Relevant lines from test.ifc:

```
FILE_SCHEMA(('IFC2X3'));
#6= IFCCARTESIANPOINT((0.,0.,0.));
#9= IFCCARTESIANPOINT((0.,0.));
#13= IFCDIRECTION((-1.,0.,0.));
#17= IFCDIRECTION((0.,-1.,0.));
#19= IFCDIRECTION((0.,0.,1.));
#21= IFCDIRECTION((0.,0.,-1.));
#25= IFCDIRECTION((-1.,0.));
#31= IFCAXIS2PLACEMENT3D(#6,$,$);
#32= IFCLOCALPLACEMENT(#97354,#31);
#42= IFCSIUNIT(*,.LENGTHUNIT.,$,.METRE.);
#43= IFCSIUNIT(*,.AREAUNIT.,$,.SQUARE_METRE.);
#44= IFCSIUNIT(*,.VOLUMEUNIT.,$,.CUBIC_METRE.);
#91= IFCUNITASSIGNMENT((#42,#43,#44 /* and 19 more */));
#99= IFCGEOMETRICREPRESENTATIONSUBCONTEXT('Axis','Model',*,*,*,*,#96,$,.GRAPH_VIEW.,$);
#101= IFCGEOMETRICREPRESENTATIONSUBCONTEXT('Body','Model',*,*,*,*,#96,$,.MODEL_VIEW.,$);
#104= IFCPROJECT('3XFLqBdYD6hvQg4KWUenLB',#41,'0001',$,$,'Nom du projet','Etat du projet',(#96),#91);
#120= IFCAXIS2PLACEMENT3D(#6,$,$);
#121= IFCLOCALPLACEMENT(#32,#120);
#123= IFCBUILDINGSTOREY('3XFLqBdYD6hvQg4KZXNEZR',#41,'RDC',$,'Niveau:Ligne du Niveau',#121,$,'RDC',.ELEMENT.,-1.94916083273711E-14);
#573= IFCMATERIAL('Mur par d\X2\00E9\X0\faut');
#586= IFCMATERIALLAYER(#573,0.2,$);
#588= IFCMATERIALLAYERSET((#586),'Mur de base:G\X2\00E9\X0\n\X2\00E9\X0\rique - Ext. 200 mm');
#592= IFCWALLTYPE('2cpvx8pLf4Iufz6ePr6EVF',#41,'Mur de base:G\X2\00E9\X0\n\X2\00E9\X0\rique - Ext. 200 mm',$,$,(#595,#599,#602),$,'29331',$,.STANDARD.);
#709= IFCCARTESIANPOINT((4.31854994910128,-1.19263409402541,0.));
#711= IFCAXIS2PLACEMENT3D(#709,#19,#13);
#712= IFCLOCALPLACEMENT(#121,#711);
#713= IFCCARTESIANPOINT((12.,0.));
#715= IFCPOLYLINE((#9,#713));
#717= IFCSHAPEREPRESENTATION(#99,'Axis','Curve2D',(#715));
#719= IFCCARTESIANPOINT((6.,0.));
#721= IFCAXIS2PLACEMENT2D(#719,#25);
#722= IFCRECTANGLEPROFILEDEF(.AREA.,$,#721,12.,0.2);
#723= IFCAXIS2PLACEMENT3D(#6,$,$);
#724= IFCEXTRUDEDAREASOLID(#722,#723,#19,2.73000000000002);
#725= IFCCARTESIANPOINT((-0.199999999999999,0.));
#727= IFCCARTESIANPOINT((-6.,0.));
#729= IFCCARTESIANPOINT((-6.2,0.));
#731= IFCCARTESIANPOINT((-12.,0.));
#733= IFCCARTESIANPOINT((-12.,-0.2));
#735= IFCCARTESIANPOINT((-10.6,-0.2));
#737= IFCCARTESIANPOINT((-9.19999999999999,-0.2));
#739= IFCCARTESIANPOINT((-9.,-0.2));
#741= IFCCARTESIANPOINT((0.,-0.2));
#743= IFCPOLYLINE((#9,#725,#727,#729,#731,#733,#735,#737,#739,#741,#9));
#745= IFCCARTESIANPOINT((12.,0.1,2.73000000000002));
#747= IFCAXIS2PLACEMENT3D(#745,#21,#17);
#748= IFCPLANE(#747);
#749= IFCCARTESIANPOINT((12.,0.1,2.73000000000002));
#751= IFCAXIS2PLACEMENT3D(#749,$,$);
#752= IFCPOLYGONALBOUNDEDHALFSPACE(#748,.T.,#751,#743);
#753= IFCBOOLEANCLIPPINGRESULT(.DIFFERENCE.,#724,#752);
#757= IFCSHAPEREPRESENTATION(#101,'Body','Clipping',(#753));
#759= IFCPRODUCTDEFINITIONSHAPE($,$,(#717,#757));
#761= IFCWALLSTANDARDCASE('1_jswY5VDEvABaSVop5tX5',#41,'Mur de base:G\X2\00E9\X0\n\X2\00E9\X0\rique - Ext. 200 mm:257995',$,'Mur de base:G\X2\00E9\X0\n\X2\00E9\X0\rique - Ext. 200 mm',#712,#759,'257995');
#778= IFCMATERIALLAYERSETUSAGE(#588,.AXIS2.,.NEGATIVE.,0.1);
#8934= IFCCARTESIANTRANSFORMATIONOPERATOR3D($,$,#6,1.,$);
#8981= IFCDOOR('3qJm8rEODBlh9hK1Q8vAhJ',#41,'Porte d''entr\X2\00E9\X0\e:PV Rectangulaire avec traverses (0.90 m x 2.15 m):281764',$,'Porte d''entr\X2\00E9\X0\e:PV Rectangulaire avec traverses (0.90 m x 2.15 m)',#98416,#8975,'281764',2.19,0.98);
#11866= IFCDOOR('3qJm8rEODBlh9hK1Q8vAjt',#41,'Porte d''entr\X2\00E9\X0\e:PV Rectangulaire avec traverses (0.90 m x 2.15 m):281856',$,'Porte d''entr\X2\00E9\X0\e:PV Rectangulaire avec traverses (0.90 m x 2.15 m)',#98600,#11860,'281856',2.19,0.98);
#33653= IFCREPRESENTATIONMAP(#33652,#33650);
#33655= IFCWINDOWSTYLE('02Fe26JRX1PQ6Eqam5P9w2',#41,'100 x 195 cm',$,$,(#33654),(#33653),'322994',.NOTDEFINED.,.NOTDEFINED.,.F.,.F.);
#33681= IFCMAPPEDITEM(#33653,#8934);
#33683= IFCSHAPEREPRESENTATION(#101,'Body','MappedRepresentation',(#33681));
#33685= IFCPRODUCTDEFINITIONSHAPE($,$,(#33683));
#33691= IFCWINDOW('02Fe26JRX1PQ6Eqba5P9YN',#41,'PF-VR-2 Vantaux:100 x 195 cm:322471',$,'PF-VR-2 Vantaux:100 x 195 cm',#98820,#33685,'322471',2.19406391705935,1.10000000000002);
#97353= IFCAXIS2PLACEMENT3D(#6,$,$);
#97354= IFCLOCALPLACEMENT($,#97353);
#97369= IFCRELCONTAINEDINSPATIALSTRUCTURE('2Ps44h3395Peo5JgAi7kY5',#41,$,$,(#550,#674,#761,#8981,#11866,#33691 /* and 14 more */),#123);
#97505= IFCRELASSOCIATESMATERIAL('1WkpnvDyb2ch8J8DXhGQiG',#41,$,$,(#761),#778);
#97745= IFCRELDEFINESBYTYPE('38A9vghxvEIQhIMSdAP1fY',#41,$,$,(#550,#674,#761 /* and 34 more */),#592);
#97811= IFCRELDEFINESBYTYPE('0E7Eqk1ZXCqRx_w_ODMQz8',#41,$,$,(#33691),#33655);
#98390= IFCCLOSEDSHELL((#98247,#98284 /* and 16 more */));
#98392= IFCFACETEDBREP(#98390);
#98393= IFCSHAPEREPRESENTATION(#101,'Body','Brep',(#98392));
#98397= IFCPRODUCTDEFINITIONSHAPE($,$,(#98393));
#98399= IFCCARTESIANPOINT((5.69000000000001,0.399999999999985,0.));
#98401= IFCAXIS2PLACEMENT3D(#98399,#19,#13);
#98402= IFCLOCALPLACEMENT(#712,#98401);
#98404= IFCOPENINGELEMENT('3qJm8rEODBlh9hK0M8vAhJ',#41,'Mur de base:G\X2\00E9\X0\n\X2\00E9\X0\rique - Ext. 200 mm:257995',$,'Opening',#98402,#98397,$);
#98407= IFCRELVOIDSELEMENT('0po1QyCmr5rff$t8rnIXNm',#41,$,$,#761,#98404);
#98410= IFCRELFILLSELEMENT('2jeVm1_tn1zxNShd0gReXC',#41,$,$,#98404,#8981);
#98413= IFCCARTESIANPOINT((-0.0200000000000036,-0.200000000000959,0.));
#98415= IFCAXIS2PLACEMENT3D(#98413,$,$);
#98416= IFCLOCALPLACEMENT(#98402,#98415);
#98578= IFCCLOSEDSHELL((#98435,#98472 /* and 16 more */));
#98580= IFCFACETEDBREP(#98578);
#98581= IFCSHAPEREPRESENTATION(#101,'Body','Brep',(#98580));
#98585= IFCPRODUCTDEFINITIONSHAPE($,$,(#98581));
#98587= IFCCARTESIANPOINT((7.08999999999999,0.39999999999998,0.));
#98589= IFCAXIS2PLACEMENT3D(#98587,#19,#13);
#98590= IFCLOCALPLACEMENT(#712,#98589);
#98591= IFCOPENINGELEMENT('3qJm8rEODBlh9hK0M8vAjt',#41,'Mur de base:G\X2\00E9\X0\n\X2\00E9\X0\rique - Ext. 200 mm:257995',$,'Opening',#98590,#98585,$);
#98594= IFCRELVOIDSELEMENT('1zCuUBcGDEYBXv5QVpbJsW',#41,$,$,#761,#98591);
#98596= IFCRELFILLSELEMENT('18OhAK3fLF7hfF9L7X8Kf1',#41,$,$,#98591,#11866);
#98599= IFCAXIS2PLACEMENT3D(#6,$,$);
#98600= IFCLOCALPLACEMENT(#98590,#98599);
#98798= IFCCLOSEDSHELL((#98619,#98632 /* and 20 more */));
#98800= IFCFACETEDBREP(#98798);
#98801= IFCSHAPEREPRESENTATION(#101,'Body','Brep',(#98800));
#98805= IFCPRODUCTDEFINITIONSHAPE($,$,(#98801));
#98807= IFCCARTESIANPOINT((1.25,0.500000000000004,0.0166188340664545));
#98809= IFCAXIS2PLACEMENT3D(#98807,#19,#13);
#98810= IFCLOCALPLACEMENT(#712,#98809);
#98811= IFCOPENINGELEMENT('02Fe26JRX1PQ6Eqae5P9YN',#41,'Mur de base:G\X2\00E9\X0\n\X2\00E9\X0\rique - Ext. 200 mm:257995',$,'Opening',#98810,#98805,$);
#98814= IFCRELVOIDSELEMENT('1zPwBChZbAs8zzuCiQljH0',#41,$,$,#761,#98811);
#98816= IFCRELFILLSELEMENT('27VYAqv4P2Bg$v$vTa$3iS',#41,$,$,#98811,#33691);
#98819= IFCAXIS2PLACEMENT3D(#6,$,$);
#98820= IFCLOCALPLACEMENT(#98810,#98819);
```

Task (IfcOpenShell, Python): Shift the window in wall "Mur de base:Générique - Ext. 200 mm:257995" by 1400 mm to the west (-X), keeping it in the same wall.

```python
import ifcopenshell
import ifcopenshell.api.geometry
import ifcopenshell.util.placement
import ifcopenshell.util.unit

model = ifcopenshell.open("test.ifc")
unit_scale = ifcopenshell.util.unit.calculate_unit_scale(model)

window = model.by_guid("02Fe26JRX1PQ6Eqba5P9YN")
opening = window.FillsVoids[0].RelatingOpeningElement
wall = opening.VoidsElements[0].RelatingBuildingElement

wall_matrix = ifcopenshell.util.placement.get_local_placement(wall.ObjectPlacement)
shift = wall_matrix[:3, 0] * 1.4 / unit_scale
before = ifcopenshell.util.placement.get_local_placement(window.ObjectPlacement)[:3, 3].copy()

# The window is placed relative to its opening, so it follows when the opening moves.
matrix = ifcopenshell.util.placement.get_local_placement(opening.ObjectPlacement)
matrix[:3, 3] += shift
ifcopenshell.api.geometry.edit_object_placement(
    model, product=opening, matrix=matrix, is_si=False, should_transform_children=True
)

after = ifcopenshell.util.placement.get_local_placement(window.ObjectPlacement)[:3, 3]
print("window moved by", (after - before).round(3) + 0.0)

model.write("test_v2.ifc")
```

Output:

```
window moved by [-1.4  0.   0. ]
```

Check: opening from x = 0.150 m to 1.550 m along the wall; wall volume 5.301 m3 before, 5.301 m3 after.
